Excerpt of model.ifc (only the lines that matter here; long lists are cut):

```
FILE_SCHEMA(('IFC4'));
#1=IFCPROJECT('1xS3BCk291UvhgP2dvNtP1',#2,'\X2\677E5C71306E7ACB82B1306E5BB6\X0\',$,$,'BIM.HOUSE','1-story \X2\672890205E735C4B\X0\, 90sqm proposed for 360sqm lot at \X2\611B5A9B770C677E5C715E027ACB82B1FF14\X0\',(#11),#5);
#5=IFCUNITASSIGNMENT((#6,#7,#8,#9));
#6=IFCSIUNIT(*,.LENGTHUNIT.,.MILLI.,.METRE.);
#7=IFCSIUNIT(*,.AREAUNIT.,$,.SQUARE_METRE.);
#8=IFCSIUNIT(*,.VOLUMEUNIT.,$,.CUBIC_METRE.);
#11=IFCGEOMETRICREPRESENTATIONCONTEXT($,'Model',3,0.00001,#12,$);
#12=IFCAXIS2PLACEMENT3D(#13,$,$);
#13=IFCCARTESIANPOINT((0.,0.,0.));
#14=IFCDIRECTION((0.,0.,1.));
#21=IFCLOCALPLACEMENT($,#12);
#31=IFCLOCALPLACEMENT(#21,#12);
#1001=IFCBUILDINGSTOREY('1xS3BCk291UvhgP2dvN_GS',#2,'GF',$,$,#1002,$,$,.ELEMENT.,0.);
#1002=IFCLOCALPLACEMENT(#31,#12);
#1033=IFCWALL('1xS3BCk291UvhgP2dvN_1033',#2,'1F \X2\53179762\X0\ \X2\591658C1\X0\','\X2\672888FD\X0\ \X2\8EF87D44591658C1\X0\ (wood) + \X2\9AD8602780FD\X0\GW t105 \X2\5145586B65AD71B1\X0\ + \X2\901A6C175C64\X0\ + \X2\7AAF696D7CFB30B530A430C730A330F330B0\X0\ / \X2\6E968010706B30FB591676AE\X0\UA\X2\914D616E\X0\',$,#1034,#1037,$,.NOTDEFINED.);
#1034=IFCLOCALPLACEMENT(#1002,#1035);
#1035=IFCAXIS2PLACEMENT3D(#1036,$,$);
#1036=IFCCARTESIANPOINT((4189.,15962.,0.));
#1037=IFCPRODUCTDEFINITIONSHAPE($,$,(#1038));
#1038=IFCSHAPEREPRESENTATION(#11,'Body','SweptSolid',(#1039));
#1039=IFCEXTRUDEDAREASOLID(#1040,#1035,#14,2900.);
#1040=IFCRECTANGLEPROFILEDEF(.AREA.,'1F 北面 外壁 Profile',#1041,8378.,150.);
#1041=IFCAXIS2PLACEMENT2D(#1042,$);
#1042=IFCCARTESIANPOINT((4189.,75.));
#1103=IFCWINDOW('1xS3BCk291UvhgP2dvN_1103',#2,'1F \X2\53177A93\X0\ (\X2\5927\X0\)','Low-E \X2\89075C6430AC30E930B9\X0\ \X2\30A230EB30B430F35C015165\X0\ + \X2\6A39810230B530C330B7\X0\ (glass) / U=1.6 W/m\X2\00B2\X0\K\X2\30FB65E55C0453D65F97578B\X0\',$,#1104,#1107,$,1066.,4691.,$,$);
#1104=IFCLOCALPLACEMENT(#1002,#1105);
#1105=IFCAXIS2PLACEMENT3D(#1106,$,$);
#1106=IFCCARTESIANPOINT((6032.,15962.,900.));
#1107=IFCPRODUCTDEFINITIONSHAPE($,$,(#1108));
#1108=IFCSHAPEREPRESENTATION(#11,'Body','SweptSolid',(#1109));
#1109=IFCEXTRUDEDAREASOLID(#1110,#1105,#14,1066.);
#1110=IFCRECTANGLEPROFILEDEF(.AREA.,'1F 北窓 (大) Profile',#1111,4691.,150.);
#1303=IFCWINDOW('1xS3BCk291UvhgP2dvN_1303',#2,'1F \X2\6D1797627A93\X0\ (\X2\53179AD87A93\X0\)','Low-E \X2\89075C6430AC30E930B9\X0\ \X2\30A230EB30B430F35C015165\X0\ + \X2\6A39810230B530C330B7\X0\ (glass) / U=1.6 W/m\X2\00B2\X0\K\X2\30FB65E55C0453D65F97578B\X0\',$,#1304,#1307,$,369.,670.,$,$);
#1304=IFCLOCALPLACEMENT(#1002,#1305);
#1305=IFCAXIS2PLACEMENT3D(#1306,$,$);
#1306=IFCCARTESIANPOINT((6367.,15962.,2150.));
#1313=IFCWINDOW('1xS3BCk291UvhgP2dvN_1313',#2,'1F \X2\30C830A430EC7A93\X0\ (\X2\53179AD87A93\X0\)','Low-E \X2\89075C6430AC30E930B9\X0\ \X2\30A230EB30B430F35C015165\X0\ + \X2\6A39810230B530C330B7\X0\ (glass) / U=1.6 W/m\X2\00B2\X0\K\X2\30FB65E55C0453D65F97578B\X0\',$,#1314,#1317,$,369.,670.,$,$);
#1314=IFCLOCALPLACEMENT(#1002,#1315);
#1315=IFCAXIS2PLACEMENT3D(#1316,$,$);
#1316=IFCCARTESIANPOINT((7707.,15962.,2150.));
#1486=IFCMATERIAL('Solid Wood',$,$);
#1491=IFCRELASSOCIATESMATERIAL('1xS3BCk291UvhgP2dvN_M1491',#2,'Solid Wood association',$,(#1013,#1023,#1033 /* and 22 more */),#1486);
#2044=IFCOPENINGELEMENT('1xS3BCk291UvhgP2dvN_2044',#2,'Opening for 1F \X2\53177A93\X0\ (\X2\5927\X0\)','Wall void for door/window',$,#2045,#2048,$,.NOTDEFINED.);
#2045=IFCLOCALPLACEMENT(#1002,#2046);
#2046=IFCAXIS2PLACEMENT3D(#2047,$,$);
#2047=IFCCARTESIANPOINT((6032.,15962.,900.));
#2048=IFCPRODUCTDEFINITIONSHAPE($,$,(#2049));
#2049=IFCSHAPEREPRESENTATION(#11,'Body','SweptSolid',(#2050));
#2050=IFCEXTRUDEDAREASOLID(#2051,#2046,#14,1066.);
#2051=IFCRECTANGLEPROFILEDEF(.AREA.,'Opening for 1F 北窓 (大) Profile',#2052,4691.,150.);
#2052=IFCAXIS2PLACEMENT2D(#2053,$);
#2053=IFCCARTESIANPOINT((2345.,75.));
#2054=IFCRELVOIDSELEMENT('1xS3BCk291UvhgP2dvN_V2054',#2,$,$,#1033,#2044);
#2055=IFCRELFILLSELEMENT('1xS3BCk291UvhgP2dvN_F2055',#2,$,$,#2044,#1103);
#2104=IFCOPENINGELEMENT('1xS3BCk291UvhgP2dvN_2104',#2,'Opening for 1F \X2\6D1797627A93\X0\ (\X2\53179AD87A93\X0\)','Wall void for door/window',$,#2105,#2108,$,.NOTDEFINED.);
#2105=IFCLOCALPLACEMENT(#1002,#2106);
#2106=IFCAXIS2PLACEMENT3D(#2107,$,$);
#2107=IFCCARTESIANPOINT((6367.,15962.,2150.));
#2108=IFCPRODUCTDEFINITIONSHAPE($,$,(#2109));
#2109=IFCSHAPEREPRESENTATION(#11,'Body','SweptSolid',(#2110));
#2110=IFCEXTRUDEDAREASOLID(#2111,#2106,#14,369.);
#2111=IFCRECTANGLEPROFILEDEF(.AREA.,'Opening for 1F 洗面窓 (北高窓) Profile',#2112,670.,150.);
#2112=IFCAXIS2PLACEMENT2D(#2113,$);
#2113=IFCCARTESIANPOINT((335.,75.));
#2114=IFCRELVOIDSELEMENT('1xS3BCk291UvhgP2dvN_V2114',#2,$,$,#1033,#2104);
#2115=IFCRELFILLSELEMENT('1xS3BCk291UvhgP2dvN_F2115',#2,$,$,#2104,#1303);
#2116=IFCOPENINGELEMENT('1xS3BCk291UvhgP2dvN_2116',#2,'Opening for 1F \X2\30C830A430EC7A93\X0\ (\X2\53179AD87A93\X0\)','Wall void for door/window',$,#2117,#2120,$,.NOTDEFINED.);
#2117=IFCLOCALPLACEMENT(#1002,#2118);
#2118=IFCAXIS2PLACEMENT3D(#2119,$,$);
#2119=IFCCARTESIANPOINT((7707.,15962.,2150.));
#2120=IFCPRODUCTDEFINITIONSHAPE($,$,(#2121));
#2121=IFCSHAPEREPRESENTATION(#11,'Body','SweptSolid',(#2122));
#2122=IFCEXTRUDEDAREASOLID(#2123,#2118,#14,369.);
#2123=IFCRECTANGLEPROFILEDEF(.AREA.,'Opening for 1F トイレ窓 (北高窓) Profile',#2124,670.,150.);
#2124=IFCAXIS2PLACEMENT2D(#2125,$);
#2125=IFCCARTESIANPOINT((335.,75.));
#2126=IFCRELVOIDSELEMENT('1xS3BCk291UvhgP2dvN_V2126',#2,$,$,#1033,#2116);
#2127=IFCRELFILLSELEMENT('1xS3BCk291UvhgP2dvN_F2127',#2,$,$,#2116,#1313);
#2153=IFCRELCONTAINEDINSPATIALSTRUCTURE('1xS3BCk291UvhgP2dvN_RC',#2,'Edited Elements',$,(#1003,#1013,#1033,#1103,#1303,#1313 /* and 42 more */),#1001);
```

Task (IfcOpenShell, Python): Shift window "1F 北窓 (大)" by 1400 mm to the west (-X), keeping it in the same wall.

```python
import ifcopenshell
import ifcopenshell.api.geometry
import ifcopenshell.util.placement
import ifcopenshell.util.unit

model = ifcopenshell.open("model.ifc")
unit_scale = ifcopenshell.util.unit.calculate_unit_scale(model)

window = model.by_guid("1xS3BCk291UvhgP2dvN_1103")
opening = window.FillsVoids[0].RelatingOpeningElement
wall = opening.VoidsElements[0].RelatingBuildingElement

wall_matrix = ifcopenshell.util.placement.get_local_placement(wall.ObjectPlacement)
shift = wall_matrix[:3, 0] * -1.4 / unit_scale
before = ifcopenshell.util.placement.get_local_placement(window.ObjectPlacement)[:3, 3].copy()

# The window is not placed relative to its opening, so move both.
for product in (opening, window):
    matrix = ifcopenshell.util.placement.get_local_placement(product.ObjectPlacement)
    matrix[:3, 3] += shift
    ifcopenshell.api.geometry.edit_object_placement(model, product=product, matrix=matrix, is_si=False)

after = ifcopenshell.util.placement.get_local_placement(window.ObjectPlacement)[:3, 3]
print("window moved by", (after - before).round(3) + 0.0)

model.write("model-out.ifc")
```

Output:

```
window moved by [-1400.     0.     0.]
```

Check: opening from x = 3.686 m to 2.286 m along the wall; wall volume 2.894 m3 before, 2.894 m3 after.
